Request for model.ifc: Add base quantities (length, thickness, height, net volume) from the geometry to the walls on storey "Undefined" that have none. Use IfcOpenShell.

First a look at what the model holds.

```python
import ifcopenshell
import ifcopenshell.util.element
import ifcopenshell.util.unit

model = ifcopenshell.open("model.ifc")
print(model.schema)
for unit_type in ("LENGTHUNIT", "AREAUNIT", "VOLUMEUNIT"):
    print(unit_type, ifcopenshell.util.unit.calculate_unit_scale(model, unit_type))
storey = next(s for s in model.by_type("IfcBuildingStorey") if s.Name == "Undefined")
walls = [e for e in ifcopenshell.util.element.get_decomposition(storey) if e.is_a("IfcWall")]
for e in sorted(walls, key=lambda e: e.id()):
    print(e.id(), e.is_a(), e.Name, list(ifcopenshell.util.element.get_psets(e, qtos_only=True)), sep=" | ")
```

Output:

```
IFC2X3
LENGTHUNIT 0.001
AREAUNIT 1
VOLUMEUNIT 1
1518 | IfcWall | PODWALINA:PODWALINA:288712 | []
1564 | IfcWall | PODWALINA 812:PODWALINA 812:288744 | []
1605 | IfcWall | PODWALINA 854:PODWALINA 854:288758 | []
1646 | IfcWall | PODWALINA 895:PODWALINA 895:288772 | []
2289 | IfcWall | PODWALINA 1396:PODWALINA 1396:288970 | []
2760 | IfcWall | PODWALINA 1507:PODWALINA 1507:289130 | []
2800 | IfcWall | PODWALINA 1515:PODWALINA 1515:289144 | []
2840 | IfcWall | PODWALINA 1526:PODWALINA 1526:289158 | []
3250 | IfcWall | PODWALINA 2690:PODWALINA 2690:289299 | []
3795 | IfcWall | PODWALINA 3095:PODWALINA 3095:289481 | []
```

```python
import ifcopenshell
import ifcopenshell.api.pset
import ifcopenshell.geom
import ifcopenshell.util.element
import ifcopenshell.util.shape
import ifcopenshell.util.unit

model = ifcopenshell.open("model.ifc")
unit_scale = ifcopenshell.util.unit.calculate_unit_scale(model)
volume_scale = ifcopenshell.util.unit.calculate_unit_scale(model, "VOLUMEUNIT")
settings = ifcopenshell.geom.settings()

storey = next(s for s in model.by_type("IfcBuildingStorey") if s.Name == "Undefined")
walls = [e for e in ifcopenshell.util.element.get_decomposition(storey) if e.is_a("IfcWall")]

for e in sorted(walls, key=lambda e: e.id()):
    if ifcopenshell.util.element.get_psets(e, qtos_only=True, should_inherit=False):
        continue
    # Geometry comes back in metres, in the element's own axes.
    shape = ifcopenshell.geom.create_shape(settings, e)
    values = {
        "Length": ifcopenshell.util.shape.get_x(shape.geometry) / unit_scale,
        "Width": ifcopenshell.util.shape.get_y(shape.geometry) / unit_scale,
        "Height": ifcopenshell.util.shape.get_z(shape.geometry) / unit_scale,
        "NetVolume": ifcopenshell.util.shape.get_volume(shape.geometry) / volume_scale,
    }
    qto = ifcopenshell.api.pset.add_qto(model, product=e, name="BaseQuantities")
    ifcopenshell.api.pset.edit_qto(model, qto=qto, properties=values)
    print(e.id(), {k: round(v, 3) for k, v in values.items()})

model.write("model_v2.ifc")
```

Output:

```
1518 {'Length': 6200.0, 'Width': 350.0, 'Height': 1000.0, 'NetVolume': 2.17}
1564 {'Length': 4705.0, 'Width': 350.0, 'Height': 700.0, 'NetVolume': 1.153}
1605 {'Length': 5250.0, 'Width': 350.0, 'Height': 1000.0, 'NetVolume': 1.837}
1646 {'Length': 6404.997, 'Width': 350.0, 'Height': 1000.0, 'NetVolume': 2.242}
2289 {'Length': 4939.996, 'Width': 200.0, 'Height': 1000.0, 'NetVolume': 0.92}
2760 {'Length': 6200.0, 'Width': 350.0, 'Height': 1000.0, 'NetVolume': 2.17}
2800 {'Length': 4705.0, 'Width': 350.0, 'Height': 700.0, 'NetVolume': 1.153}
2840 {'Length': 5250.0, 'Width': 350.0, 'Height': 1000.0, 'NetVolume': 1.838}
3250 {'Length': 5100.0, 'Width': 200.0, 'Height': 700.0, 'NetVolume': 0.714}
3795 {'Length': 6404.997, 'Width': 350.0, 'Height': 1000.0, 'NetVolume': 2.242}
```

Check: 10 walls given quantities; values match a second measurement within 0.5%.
